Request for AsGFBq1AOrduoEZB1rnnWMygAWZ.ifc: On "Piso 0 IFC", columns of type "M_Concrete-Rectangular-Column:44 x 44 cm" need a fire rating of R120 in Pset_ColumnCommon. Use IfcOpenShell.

First a look at what the model holds.

```python
import ifcopenshell
import ifcopenshell.util.element

model = ifcopenshell.open("AsGFBq1AOrduoEZB1rnnWMygAWZ.ifc")
print(model.schema)
storey = next(s for s in model.by_type("IfcBuildingStorey") if s.Name == "Piso 0 IFC")
columns = [e for e in ifcopenshell.util.element.get_decomposition(storey) if e.is_a("IfcColumn")]
seen = {}
for e in columns:
    element_type = ifcopenshell.util.element.get_type(e)
    key = (element_type.Name if element_type != e and element_type else None, ifcopenshell.util.element.get_pset(e, "Pset_ColumnCommon", "FireRating"))
    seen[key] = seen.get(key, 0) + 1
for (name, value), count in sorted(seen.items(), key=str):
    print(count, "x", name, "|", value)
```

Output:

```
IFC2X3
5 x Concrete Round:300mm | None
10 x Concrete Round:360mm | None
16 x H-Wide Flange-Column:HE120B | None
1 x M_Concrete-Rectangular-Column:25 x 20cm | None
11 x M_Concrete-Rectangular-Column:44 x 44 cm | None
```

```python
import ifcopenshell
import ifcopenshell.api.pset
import ifcopenshell.util.element

model = ifcopenshell.open("AsGFBq1AOrduoEZB1rnnWMygAWZ.ifc")

storey = next(s for s in model.by_type("IfcBuildingStorey") if s.Name == "Piso 0 IFC")
columns = [e for e in ifcopenshell.util.element.get_decomposition(storey) if e.is_a("IfcColumn")]

count = 0
for e in columns:
    element_type = ifcopenshell.util.element.get_type(e)
    if element_type in (None, e) or element_type.Name != "M_Concrete-Rectangular-Column:44 x 44 cm":
        continue
    # add_pset returns the element's existing set when there is one.
    pset = ifcopenshell.api.pset.add_pset(model, product=e, name="Pset_ColumnCommon")
    ifcopenshell.api.pset.edit_pset(model, pset=pset, properties={"FireRating": "R120"})
    count += 1

print(count, "columns updated")

model.write("AsGFBq1AOrduoEZB1rnnWMygAWZ_rev.ifc")
```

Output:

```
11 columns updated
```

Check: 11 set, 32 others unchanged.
